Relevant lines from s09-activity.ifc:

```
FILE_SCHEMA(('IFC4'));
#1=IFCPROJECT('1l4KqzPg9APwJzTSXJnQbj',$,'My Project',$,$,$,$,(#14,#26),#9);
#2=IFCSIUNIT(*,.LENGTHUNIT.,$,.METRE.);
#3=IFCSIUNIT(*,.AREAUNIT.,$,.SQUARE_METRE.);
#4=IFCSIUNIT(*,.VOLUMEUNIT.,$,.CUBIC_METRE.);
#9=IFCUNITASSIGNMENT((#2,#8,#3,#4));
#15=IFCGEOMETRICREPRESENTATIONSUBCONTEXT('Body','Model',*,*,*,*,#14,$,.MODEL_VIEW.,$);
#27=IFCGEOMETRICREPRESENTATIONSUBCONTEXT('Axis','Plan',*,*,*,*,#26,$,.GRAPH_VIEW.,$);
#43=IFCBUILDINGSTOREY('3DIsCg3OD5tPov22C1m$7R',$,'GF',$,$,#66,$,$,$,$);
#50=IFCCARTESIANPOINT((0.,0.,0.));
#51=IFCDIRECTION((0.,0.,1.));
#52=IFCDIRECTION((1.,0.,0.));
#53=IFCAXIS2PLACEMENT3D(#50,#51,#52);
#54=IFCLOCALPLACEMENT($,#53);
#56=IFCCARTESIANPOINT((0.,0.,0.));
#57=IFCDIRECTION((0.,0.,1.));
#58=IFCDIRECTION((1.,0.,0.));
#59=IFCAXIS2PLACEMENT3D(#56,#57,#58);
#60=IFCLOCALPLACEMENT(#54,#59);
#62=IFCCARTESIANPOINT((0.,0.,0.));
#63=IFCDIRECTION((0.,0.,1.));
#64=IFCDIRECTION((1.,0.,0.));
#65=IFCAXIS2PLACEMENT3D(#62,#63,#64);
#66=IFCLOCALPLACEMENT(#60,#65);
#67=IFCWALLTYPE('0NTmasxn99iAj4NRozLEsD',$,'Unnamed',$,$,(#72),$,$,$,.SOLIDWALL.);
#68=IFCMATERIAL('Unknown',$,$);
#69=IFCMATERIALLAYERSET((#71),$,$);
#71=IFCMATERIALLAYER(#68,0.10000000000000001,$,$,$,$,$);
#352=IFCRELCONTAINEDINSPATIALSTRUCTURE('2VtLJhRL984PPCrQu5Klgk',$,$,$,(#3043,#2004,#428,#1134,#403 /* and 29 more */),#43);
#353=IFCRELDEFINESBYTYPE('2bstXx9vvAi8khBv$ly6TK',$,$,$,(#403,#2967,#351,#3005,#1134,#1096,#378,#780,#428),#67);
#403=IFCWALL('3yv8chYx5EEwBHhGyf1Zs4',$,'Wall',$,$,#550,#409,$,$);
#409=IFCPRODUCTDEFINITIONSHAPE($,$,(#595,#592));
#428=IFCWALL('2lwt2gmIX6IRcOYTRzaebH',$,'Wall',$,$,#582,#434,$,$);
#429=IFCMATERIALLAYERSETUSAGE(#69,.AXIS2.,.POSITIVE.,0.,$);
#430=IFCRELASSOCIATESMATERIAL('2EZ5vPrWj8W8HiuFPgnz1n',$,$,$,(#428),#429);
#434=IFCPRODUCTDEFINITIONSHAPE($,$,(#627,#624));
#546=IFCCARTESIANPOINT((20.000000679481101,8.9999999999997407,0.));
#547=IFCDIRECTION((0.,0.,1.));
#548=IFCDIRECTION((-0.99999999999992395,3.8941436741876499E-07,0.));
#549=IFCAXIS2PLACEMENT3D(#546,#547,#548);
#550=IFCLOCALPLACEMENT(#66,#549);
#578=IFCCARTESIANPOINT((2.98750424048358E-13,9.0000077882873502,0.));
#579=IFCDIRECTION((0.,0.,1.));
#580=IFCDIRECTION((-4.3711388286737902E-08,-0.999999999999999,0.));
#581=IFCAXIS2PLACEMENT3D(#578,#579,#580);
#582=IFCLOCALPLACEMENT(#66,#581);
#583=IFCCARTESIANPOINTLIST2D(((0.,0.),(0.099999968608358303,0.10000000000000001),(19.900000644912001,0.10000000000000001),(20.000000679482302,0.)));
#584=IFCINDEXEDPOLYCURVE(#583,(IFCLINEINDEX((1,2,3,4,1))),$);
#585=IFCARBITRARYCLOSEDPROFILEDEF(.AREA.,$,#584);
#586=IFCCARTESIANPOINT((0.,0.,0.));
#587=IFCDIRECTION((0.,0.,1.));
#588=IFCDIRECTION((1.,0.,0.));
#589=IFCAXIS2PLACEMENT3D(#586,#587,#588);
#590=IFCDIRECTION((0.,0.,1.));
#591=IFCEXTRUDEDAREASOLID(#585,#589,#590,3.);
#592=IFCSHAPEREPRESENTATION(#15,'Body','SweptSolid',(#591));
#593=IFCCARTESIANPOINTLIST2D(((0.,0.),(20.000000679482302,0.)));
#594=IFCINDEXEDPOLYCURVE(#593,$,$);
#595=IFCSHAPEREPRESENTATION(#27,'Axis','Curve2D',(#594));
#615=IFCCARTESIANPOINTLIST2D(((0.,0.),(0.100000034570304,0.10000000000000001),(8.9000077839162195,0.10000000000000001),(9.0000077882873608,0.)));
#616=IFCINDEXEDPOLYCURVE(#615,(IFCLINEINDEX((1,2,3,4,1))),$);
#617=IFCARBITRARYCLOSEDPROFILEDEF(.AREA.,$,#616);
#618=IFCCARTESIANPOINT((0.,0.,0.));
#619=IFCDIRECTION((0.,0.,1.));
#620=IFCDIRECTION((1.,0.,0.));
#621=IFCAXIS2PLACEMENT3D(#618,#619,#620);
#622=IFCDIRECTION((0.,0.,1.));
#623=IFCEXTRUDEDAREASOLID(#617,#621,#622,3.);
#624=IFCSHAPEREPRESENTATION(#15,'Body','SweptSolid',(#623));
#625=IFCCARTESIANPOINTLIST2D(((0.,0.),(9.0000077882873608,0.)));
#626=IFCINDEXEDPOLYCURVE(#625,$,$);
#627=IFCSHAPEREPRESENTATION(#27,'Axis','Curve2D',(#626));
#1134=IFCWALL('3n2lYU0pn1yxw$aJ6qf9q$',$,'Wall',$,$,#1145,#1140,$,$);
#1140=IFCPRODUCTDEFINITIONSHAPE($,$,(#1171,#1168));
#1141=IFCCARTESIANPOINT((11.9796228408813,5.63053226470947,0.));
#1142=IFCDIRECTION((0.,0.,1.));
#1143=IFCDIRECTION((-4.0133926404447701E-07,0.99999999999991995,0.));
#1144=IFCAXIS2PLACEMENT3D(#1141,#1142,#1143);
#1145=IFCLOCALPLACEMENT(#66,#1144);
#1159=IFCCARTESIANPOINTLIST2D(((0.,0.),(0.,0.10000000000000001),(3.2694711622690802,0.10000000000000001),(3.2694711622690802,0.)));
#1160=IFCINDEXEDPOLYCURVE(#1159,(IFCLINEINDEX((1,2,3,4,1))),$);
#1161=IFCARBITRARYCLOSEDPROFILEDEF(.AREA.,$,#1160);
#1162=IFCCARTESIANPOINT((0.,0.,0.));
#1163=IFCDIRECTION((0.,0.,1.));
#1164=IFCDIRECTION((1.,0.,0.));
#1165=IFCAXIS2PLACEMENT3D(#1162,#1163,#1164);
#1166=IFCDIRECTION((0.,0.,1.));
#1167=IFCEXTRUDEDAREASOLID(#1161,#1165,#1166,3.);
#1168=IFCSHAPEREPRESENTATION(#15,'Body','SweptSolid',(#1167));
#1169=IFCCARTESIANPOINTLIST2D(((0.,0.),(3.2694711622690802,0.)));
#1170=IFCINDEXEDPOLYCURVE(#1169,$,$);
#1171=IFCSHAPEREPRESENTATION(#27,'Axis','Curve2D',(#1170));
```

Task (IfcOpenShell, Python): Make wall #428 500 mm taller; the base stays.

```python
import ifcopenshell
import ifcopenshell.geom
import ifcopenshell.util.representation
import ifcopenshell.util.shape
import ifcopenshell.util.unit

model = ifcopenshell.open("s09-activity.ifc")
unit_scale = ifcopenshell.util.unit.calculate_unit_scale(model)
settings = ifcopenshell.geom.settings()


def volume(element):
    """Net volume in cubic metres, openings subtracted."""
    shape = ifcopenshell.geom.create_shape(settings, element)
    return ifcopenshell.util.shape.get_volume(shape.geometry)


wall = model.by_id(428)
before = volume(wall)

body = ifcopenshell.util.representation.get_representation(wall, "Model", "Body")
solid = body.Items[0]
old_height = solid.Depth
solid.Depth += 0.5 / unit_scale
after = volume(wall)

print(f"height {old_height:g} -> {solid.Depth:g}, volume {before:.3f} -> {after:.3f} m3")

model.write("s09-activity_rev.ifc")
```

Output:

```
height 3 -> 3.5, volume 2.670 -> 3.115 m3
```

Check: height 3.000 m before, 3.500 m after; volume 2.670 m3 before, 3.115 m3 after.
